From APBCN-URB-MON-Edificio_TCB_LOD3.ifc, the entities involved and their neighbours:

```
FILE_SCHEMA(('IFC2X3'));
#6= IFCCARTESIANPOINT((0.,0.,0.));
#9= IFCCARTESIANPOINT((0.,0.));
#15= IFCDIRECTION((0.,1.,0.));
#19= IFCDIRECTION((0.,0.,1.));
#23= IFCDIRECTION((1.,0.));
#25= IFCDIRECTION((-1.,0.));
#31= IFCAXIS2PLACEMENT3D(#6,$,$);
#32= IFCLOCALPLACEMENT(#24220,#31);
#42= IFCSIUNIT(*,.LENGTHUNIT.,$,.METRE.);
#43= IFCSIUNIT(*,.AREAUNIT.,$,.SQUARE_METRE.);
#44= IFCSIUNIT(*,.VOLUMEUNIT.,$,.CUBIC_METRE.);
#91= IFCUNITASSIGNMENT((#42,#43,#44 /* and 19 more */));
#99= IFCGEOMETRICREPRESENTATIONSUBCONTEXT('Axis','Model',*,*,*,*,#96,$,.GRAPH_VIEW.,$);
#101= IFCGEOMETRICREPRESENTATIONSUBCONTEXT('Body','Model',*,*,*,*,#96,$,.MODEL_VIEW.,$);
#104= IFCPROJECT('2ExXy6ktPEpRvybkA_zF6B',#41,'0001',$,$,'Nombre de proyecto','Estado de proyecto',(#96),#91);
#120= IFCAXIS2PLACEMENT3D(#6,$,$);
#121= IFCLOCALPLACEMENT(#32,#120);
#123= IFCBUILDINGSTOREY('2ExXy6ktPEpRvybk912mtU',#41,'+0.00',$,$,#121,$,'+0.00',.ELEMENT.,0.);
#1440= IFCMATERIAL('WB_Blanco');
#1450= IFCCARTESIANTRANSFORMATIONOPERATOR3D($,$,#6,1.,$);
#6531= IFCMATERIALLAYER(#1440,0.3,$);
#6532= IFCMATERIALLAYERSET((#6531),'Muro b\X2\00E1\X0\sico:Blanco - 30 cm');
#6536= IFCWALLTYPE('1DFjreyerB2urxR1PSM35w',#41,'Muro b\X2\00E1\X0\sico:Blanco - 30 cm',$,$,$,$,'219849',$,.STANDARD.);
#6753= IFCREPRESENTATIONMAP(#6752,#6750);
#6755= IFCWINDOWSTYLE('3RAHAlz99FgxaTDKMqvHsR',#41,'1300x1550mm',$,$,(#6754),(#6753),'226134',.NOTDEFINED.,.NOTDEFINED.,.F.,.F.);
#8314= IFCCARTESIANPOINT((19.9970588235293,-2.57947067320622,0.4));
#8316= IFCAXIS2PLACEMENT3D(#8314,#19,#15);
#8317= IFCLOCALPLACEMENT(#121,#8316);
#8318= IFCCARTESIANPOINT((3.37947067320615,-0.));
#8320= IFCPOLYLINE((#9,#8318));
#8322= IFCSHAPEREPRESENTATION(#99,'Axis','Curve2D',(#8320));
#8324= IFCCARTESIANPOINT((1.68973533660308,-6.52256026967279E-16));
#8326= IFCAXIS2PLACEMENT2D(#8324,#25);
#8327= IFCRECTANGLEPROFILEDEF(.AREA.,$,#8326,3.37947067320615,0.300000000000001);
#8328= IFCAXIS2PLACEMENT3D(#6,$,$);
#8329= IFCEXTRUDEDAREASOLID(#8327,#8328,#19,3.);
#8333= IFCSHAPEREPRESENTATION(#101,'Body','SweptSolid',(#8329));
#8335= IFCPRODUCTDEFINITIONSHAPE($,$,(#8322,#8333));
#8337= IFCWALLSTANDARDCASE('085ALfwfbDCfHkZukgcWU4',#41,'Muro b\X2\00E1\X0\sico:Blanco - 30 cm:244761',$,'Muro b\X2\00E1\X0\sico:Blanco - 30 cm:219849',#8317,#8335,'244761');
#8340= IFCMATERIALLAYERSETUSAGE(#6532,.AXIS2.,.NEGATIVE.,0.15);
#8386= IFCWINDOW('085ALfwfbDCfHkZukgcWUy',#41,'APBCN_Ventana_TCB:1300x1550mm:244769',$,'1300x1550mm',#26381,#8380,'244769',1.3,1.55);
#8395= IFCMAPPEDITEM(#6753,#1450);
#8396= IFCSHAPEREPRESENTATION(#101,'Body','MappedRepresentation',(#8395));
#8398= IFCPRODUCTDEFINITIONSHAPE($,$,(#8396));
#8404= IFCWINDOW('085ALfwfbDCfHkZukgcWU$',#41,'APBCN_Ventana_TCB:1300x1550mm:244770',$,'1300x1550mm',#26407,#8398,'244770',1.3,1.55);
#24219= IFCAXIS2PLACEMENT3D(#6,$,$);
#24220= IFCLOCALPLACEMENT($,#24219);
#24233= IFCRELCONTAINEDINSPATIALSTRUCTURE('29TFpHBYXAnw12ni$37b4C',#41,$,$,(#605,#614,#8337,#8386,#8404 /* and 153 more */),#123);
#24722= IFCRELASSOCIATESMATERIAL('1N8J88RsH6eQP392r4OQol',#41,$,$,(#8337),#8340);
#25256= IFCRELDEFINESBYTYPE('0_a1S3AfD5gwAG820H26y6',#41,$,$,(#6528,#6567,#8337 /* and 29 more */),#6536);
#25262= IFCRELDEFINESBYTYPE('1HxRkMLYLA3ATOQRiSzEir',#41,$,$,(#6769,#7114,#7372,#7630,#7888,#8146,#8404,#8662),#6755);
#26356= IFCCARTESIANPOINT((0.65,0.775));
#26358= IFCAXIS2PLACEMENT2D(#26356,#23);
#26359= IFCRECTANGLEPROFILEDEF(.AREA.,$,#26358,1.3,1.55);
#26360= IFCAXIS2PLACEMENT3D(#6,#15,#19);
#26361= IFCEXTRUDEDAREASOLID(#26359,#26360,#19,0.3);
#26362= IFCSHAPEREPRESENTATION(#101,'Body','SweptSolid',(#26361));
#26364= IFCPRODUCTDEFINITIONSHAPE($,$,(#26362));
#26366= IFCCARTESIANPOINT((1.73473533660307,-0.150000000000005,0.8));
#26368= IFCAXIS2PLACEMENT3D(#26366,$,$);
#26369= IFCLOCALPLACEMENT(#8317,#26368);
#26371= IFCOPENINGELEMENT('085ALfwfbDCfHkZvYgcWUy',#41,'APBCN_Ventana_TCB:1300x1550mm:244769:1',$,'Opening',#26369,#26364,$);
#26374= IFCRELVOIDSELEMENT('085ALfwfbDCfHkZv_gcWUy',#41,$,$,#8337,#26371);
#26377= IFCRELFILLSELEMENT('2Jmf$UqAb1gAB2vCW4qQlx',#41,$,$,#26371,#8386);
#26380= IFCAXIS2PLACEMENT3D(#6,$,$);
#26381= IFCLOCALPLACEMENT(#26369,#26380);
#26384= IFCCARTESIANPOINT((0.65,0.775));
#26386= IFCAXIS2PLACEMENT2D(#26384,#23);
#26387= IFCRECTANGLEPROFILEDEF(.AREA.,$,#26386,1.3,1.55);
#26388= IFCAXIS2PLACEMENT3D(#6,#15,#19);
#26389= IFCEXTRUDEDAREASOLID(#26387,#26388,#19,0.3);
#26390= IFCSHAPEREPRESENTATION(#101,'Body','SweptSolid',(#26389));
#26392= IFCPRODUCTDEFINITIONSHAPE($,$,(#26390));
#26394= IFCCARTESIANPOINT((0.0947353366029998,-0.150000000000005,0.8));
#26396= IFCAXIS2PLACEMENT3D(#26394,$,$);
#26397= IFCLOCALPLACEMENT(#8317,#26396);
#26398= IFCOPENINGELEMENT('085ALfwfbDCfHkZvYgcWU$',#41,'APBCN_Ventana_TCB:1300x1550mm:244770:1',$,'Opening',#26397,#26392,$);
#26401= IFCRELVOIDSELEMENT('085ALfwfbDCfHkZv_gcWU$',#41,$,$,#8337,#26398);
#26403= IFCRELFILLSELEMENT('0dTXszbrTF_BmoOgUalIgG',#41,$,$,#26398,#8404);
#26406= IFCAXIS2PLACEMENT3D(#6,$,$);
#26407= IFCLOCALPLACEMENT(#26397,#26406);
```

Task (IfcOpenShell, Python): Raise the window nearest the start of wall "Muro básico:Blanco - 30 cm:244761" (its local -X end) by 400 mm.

```python
import numpy as np
import ifcopenshell
import ifcopenshell.api.geometry
import ifcopenshell.util.placement
import ifcopenshell.util.unit

model = ifcopenshell.open("APBCN-URB-MON-Edificio_TCB_LOD3.ifc")
unit_scale = ifcopenshell.util.unit.calculate_unit_scale(model)

window = model.by_id(8404)
opening = window.FillsVoids[0].RelatingOpeningElement
dz = 0.4

shift = np.array([0.0, 0.0, dz])
# The window is placed relative to its opening, so it follows when the opening moves.
matrix = ifcopenshell.util.placement.get_local_placement(opening.ObjectPlacement)
matrix[:3, 3] += shift
ifcopenshell.api.geometry.edit_object_placement(
    model, product=opening, matrix=matrix, is_si=False, should_transform_children=True
)

print(f"moved by {dz * unit_scale:+.3f} m")

model.write("APBCN-URB-MON-Edificio_TCB_LOD3_updated.ifc")
```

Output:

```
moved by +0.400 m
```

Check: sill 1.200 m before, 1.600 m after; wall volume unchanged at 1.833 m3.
